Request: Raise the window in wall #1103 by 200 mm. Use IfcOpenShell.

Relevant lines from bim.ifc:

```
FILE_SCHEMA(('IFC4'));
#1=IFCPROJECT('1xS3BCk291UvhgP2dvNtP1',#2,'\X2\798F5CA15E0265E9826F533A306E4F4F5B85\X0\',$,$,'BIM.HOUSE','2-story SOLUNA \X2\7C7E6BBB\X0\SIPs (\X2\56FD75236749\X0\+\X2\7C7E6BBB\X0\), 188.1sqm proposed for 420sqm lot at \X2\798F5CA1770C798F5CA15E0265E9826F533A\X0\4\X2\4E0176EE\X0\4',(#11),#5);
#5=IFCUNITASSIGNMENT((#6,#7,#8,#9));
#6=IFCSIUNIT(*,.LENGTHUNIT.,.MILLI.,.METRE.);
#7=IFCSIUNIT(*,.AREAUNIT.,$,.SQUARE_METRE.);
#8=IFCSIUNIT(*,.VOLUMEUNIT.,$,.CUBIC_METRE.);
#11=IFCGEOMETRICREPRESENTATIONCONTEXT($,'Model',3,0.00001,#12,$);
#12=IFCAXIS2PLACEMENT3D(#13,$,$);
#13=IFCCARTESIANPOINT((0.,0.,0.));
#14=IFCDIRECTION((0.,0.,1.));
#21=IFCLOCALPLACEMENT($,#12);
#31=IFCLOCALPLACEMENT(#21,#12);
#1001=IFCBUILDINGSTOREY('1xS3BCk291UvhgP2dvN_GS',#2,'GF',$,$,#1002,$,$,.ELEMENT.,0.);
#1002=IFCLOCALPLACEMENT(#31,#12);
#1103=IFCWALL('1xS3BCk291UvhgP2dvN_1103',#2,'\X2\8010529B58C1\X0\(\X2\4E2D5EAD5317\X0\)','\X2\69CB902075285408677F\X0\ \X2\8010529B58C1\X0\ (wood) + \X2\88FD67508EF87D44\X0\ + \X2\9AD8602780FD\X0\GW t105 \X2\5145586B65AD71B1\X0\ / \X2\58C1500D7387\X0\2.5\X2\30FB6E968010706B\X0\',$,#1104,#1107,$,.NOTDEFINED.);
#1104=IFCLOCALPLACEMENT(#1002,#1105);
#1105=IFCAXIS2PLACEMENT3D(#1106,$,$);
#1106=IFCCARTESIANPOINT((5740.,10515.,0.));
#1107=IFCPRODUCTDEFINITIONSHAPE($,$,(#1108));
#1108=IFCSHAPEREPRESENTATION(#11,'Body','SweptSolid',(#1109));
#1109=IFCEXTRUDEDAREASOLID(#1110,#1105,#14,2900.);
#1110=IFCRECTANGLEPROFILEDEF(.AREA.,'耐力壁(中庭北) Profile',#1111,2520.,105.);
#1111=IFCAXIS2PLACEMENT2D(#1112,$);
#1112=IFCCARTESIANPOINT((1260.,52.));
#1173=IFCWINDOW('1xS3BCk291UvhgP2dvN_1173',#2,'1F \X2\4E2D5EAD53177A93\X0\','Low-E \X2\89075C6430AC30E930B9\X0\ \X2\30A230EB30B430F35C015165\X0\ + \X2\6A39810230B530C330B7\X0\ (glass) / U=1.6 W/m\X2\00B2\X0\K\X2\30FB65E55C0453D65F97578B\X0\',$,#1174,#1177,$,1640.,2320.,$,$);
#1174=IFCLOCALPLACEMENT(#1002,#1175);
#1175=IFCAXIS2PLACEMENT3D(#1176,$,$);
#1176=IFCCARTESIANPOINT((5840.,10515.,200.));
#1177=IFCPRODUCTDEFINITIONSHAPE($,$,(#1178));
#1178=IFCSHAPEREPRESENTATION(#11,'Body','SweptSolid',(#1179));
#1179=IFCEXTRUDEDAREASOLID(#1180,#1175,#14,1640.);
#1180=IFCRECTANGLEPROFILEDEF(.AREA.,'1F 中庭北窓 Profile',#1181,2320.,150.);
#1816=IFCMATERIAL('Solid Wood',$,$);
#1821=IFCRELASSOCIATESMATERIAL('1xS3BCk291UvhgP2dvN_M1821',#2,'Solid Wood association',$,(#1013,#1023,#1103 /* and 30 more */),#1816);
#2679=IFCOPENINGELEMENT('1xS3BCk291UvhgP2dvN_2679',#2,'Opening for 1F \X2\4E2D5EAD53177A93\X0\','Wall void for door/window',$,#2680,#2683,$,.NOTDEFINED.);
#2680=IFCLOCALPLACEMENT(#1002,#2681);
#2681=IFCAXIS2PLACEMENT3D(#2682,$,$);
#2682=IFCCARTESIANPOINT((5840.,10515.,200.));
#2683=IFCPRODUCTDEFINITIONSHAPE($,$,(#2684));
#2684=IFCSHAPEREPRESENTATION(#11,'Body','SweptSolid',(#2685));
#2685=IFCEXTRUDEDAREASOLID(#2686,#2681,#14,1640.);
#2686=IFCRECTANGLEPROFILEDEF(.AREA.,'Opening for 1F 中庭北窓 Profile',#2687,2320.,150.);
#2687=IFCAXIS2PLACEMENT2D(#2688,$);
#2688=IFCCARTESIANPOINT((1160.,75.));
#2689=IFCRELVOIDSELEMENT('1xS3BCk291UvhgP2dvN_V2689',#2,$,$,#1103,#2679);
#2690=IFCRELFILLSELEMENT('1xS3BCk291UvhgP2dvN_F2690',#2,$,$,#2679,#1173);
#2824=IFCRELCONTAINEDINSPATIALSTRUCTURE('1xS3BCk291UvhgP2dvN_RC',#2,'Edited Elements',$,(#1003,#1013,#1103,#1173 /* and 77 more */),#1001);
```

```python
import numpy as np
import ifcopenshell
import ifcopenshell.api.geometry
import ifcopenshell.util.placement
import ifcopenshell.util.unit

model = ifcopenshell.open("bim.ifc")
unit_scale = ifcopenshell.util.unit.calculate_unit_scale(model)

window = model.by_guid("1xS3BCk291UvhgP2dvN_1173")
opening = window.FillsVoids[0].RelatingOpeningElement
dz = 0.2 / unit_scale

shift = np.array([0.0, 0.0, dz])
# The window is not placed relative to its opening, so move both.
for product in (opening, window):
    matrix = ifcopenshell.util.placement.get_local_placement(product.ObjectPlacement)
    matrix[:3, 3] += shift
    ifcopenshell.api.geometry.edit_object_placement(model, product=product, matrix=matrix, is_si=False)

print(f"moved by {dz * unit_scale:+.3f} m")

model.write("bim_updated.ifc")
```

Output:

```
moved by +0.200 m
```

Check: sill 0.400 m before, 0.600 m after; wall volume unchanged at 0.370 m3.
